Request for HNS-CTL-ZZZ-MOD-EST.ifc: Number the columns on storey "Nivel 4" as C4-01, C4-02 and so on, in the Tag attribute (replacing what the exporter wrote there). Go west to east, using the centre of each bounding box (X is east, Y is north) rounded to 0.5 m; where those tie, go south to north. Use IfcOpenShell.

First a look at what the model holds.

```python
import ifcopenshell
import ifcopenshell.util.element
import ifcopenshell.util.placement

model = ifcopenshell.open("HNS-CTL-ZZZ-MOD-EST.ifc")
print(model.schema)
storey = next(s for s in model.by_type("IfcBuildingStorey") if s.Name == "Nivel 4")
columns = [e for e in ifcopenshell.util.element.get_decomposition(storey) if e.is_a("IfcColumn")]
for e in sorted(columns, key=lambda e: e.id()):
    origin = ifcopenshell.util.placement.get_local_placement(e.ObjectPlacement)[:3, 3]
    print(e.id(), e.Tag, e.Name, origin.round(2) + 0.0, sep=" | ")
```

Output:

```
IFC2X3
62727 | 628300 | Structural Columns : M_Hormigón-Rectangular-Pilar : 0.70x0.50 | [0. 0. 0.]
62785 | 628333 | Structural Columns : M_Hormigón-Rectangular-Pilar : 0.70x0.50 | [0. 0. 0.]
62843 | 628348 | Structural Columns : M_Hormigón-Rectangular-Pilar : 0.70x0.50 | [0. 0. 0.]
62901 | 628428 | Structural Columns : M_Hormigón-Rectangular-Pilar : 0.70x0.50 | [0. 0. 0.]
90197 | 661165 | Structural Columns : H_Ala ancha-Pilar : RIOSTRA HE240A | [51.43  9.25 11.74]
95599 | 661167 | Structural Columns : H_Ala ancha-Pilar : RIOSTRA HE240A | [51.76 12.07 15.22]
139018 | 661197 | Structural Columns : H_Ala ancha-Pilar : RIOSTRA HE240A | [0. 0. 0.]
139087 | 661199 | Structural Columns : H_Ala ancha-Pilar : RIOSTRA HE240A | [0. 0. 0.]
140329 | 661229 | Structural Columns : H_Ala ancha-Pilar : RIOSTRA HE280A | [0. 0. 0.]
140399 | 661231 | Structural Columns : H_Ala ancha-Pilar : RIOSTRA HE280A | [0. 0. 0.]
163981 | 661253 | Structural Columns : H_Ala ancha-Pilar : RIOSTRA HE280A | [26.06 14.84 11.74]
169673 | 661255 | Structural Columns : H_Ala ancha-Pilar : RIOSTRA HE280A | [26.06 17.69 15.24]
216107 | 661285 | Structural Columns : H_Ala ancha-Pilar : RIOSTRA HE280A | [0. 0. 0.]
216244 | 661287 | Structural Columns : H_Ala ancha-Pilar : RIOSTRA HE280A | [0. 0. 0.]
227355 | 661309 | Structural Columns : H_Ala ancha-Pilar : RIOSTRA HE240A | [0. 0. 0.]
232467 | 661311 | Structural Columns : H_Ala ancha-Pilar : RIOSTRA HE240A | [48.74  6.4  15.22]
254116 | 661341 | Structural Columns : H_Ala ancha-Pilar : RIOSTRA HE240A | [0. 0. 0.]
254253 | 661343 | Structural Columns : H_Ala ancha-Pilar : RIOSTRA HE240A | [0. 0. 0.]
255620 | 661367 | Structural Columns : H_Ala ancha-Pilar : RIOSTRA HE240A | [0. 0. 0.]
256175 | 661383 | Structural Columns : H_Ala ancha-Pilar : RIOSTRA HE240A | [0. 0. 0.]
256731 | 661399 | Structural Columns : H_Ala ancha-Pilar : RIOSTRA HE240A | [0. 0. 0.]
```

```python
import ifcopenshell
import ifcopenshell.geom
import ifcopenshell.util.element
import ifcopenshell.util.shape

model = ifcopenshell.open("HNS-CTL-ZZZ-MOD-EST.ifc")
settings = ifcopenshell.geom.settings()
settings.set("use-world-coords", True)


def centre(element):
    shape = ifcopenshell.geom.create_shape(settings, element)
    return ifcopenshell.util.shape.get_bbox_centroid(shape.geometry)


storey = next(s for s in model.by_type("IfcBuildingStorey") if s.Name == "Nivel 4")
columns = [e for e in ifcopenshell.util.element.get_decomposition(storey) if e.is_a("IfcColumn")]

# Insertion points can sit at a corner or the storey origin, so sort by the geometry (in metres).
centres = {e: centre(e) for e in columns}
columns.sort(key=lambda e: (round(centres[e][0] / 0.5), centres[e][1]))

for i, e in enumerate(columns, start=1):
    number = f"C4-{i:02d}"
    e.Tag = number
    print(e.id(), number)

model.write("HNS-CTL-ZZZ-MOD-EST_rev.ifc")
```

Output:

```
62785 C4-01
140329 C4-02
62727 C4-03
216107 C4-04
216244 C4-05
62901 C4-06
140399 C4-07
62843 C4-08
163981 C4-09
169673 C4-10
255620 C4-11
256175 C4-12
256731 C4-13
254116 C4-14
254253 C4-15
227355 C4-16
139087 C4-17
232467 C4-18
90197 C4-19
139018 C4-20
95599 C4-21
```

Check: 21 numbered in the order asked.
